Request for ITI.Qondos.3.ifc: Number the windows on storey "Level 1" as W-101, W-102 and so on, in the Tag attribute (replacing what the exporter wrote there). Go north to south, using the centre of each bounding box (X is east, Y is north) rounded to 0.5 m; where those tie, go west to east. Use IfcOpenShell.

First a look at what the model holds.

```python
import ifcopenshell
import ifcopenshell.util.element
import ifcopenshell.util.placement

model = ifcopenshell.open("ITI.Qondos.3.ifc")
print(model.schema)
storey = next(s for s in model.by_type("IfcBuildingStorey") if s.Name == "Level 1")
windows = [e for e in ifcopenshell.util.element.get_decomposition(storey) if e.is_a("IfcWindow")]
for e in sorted(windows, key=lambda e: e.id()):
    origin = ifcopenshell.util.placement.get_local_placement(e.ObjectPlacement)[:3, 3]
    print(e.id(), e.Tag, e.Name, origin.round(2) + 0.0, sep=" | ")
```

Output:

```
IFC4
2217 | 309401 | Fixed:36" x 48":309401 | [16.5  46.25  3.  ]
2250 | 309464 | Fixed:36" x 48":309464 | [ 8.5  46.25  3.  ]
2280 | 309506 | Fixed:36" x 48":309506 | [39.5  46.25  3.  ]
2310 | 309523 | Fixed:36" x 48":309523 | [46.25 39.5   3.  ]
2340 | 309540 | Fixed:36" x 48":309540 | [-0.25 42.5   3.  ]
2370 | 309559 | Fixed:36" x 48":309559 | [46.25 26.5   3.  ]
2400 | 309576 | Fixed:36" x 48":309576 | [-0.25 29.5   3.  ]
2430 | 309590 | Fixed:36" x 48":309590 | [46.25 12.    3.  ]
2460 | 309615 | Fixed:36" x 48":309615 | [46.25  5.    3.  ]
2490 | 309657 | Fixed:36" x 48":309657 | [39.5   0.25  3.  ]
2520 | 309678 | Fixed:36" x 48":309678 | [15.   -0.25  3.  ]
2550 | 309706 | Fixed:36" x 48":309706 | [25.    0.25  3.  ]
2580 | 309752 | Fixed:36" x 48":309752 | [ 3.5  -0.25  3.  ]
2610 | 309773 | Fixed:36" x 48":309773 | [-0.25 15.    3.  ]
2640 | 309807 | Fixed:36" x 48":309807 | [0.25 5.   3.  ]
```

```python
import ifcopenshell
import ifcopenshell.geom
import ifcopenshell.util.element
import ifcopenshell.util.shape

model = ifcopenshell.open("ITI.Qondos.3.ifc")
settings = ifcopenshell.geom.settings()
settings.set("use-world-coords", True)


def centre(element):
    shape = ifcopenshell.geom.create_shape(settings, element)
    return ifcopenshell.util.shape.get_bbox_centroid(shape.geometry)


storey = next(s for s in model.by_type("IfcBuildingStorey") if s.Name == "Level 1")
windows = [e for e in ifcopenshell.util.element.get_decomposition(storey) if e.is_a("IfcWindow")]

# Insertion points can sit at a corner or the storey origin, so sort by the geometry (in metres).
centres = {e: centre(e) for e in windows}
windows.sort(key=lambda e: (-round(centres[e][1] / 0.5), centres[e][0]))

for i, e in enumerate(windows, start=1):
    number = f"W-1{i:02d}"
    e.Tag = number
    print(e.id(), number)

model.write("ITI.Qondos.3_rev.ifc")
```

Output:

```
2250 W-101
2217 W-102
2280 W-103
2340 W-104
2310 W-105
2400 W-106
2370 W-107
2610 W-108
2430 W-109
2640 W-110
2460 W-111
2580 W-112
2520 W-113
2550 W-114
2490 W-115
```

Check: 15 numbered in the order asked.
